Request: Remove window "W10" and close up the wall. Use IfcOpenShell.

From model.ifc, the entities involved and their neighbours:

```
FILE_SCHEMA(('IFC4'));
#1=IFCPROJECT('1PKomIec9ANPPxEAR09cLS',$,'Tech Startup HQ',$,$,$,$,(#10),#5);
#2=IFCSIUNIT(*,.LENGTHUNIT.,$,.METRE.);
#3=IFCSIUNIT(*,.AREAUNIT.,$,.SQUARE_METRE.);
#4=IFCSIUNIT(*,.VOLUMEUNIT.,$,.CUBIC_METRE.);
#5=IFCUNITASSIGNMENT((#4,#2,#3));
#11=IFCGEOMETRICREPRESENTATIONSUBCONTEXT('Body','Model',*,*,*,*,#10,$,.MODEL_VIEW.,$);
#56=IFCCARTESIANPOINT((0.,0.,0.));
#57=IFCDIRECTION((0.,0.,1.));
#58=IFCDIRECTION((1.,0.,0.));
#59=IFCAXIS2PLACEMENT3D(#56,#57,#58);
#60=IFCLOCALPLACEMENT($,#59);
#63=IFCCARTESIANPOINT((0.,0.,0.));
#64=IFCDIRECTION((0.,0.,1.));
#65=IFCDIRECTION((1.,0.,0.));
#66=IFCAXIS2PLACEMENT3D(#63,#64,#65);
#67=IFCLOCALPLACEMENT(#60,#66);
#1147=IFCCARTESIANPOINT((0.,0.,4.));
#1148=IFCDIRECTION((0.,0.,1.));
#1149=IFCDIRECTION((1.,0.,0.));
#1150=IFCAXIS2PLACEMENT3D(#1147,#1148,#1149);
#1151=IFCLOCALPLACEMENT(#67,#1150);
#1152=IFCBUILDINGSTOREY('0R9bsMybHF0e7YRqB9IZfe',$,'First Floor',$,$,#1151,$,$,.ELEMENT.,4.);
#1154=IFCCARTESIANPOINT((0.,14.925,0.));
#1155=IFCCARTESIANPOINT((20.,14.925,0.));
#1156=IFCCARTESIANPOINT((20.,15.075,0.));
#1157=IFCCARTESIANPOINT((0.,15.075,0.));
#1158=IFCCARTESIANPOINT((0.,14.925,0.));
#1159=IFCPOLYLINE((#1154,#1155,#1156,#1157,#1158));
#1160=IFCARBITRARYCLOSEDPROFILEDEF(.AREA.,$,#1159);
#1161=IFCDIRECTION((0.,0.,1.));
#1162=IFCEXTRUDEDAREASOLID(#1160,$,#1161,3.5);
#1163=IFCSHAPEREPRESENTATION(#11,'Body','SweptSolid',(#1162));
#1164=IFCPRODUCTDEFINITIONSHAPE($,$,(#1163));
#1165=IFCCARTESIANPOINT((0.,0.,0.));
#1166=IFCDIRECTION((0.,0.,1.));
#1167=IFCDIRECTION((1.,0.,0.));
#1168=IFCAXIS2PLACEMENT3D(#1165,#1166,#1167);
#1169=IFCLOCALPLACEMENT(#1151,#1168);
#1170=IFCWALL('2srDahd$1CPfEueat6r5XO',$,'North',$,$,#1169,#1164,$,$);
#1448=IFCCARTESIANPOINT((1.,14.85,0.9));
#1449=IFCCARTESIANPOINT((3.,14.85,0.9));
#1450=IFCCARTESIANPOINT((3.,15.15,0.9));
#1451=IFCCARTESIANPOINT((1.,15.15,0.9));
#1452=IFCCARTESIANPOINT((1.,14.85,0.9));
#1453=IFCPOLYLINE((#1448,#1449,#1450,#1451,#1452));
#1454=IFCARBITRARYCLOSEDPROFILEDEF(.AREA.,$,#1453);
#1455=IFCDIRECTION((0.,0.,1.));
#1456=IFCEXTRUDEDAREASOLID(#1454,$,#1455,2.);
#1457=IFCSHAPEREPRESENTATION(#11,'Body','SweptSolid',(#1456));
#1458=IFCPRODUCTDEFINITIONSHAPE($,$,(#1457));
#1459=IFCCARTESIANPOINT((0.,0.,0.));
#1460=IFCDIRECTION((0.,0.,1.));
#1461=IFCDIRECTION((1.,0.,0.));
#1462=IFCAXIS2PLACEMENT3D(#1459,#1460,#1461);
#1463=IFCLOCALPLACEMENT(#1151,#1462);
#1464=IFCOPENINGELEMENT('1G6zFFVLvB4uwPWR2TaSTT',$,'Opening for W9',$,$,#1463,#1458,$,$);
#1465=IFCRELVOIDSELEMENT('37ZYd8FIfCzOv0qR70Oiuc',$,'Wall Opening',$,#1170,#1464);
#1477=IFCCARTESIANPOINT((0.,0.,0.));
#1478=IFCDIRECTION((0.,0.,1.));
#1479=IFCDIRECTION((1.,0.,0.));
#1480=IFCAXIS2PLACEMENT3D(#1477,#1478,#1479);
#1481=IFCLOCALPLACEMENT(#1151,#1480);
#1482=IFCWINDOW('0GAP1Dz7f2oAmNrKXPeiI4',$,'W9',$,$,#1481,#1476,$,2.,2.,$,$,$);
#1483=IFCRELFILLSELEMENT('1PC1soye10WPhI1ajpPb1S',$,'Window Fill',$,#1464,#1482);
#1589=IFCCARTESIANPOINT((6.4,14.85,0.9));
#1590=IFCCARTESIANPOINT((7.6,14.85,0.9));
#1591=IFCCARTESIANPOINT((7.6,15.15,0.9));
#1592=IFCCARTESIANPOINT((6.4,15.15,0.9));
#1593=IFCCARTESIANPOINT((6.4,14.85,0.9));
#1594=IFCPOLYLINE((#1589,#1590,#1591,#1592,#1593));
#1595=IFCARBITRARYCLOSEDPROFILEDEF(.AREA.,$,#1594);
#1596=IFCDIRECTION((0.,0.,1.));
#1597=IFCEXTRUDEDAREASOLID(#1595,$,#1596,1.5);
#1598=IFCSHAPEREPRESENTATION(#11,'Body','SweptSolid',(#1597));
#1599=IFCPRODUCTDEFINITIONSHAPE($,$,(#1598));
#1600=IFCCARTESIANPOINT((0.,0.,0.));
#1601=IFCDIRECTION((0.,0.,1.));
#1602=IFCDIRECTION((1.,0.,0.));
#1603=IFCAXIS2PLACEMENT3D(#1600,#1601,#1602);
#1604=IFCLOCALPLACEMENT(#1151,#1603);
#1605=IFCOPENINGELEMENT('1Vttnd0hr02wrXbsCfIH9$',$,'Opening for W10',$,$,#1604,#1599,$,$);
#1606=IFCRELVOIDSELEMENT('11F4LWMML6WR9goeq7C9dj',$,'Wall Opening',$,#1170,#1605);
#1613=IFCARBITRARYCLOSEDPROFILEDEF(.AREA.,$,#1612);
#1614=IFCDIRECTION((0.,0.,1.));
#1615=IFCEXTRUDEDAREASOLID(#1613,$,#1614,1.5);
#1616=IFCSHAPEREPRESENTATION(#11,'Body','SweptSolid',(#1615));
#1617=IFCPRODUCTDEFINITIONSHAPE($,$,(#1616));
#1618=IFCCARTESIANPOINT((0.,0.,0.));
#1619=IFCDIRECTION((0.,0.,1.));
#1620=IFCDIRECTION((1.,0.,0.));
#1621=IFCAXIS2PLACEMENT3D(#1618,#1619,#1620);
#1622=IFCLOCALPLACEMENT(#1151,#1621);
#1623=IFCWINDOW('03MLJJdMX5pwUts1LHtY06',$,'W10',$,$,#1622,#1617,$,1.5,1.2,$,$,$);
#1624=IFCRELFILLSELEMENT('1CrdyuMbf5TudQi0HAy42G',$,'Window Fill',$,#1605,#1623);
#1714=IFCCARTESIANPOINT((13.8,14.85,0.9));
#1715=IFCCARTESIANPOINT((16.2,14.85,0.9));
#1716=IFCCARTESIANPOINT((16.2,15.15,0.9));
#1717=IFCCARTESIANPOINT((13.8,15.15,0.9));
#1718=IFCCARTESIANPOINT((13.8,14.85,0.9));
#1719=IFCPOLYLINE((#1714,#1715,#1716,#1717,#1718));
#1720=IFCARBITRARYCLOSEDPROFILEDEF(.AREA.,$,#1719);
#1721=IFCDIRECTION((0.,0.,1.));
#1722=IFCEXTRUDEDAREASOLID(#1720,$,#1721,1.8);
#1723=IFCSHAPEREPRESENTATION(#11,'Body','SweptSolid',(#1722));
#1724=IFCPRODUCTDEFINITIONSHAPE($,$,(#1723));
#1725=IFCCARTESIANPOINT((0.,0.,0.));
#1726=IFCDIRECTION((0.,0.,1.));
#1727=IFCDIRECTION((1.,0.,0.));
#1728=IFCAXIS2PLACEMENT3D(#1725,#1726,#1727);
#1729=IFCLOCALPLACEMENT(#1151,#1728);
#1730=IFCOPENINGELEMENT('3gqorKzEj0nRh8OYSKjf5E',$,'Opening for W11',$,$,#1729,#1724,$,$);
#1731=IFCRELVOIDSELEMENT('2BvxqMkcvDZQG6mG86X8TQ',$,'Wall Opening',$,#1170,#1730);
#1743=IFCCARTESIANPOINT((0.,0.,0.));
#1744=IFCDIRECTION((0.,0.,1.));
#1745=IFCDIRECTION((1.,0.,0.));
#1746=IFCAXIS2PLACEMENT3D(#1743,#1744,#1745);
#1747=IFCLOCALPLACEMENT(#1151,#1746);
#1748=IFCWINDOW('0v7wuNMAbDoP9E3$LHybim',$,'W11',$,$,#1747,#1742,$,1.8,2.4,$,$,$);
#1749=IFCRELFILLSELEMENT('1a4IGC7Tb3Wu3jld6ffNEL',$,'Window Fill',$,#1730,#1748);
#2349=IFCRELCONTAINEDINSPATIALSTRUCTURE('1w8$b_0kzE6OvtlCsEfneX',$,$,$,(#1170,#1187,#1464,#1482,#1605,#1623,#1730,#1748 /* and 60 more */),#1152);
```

```python
import ifcopenshell
import ifcopenshell.api.feature
import ifcopenshell.api.root
import ifcopenshell.geom
import ifcopenshell.util.shape

model = ifcopenshell.open("model.ifc")
settings = ifcopenshell.geom.settings()


def volume(element):
    """Net volume in cubic metres, openings subtracted."""
    shape = ifcopenshell.geom.create_shape(settings, element)
    return ifcopenshell.util.shape.get_volume(shape.geometry)


window = model.by_id(1623)
opening = window.FillsVoids[0].RelatingOpeningElement
wall = opening.VoidsElements[0].RelatingBuildingElement
before = volume(wall)

ifcopenshell.api.root.remove_product(model, product=window)
ifcopenshell.api.feature.remove_feature(model, feature=opening)

after = volume(wall)

print(f"wall volume {before:.3f} -> {after:.3f} m3")

model.write("model_updated.ifc")
```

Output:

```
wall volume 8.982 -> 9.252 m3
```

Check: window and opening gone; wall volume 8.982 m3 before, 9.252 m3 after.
